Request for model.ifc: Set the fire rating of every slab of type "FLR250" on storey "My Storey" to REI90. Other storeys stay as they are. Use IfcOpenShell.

First a look at what the model holds.

```python
import ifcopenshell
import ifcopenshell.util.element

model = ifcopenshell.open("model.ifc")
print(model.schema)
storey = next(s for s in model.by_type("IfcBuildingStorey") if s.Name == "My Storey")
slabs = [e for e in ifcopenshell.util.element.get_decomposition(storey) if e.is_a("IfcSlab")]
seen = {}
for e in slabs:
    element_type = ifcopenshell.util.element.get_type(e)
    key = (element_type.Name if element_type != e and element_type else None, ifcopenshell.util.element.get_pset(e, "Pset_SlabCommon", "FireRating"))
    seen[key] = seen.get(key, 0) + 1
for (name, value), count in sorted(seen.items(), key=str):
    print(count, "x", name, "|", value)
```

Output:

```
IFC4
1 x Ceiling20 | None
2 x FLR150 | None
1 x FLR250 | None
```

```python
import ifcopenshell
import ifcopenshell.api.pset
import ifcopenshell.util.element

model = ifcopenshell.open("model.ifc")

storey = next(s for s in model.by_type("IfcBuildingStorey") if s.Name == "My Storey")
slabs = [e for e in ifcopenshell.util.element.get_decomposition(storey) if e.is_a("IfcSlab")]

count = 0
for e in slabs:
    element_type = ifcopenshell.util.element.get_type(e)
    if element_type in (None, e) or element_type.Name != "FLR250":
        continue
    # add_pset returns the element's existing set when there is one.
    pset = ifcopenshell.api.pset.add_pset(model, product=e, name="Pset_SlabCommon")
    ifcopenshell.api.pset.edit_pset(model, pset=pset, properties={"FireRating": "REI90"})
    count += 1

print(count, "slabs updated")

model.write("model_rev.ifc")
```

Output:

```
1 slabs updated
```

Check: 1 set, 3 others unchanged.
